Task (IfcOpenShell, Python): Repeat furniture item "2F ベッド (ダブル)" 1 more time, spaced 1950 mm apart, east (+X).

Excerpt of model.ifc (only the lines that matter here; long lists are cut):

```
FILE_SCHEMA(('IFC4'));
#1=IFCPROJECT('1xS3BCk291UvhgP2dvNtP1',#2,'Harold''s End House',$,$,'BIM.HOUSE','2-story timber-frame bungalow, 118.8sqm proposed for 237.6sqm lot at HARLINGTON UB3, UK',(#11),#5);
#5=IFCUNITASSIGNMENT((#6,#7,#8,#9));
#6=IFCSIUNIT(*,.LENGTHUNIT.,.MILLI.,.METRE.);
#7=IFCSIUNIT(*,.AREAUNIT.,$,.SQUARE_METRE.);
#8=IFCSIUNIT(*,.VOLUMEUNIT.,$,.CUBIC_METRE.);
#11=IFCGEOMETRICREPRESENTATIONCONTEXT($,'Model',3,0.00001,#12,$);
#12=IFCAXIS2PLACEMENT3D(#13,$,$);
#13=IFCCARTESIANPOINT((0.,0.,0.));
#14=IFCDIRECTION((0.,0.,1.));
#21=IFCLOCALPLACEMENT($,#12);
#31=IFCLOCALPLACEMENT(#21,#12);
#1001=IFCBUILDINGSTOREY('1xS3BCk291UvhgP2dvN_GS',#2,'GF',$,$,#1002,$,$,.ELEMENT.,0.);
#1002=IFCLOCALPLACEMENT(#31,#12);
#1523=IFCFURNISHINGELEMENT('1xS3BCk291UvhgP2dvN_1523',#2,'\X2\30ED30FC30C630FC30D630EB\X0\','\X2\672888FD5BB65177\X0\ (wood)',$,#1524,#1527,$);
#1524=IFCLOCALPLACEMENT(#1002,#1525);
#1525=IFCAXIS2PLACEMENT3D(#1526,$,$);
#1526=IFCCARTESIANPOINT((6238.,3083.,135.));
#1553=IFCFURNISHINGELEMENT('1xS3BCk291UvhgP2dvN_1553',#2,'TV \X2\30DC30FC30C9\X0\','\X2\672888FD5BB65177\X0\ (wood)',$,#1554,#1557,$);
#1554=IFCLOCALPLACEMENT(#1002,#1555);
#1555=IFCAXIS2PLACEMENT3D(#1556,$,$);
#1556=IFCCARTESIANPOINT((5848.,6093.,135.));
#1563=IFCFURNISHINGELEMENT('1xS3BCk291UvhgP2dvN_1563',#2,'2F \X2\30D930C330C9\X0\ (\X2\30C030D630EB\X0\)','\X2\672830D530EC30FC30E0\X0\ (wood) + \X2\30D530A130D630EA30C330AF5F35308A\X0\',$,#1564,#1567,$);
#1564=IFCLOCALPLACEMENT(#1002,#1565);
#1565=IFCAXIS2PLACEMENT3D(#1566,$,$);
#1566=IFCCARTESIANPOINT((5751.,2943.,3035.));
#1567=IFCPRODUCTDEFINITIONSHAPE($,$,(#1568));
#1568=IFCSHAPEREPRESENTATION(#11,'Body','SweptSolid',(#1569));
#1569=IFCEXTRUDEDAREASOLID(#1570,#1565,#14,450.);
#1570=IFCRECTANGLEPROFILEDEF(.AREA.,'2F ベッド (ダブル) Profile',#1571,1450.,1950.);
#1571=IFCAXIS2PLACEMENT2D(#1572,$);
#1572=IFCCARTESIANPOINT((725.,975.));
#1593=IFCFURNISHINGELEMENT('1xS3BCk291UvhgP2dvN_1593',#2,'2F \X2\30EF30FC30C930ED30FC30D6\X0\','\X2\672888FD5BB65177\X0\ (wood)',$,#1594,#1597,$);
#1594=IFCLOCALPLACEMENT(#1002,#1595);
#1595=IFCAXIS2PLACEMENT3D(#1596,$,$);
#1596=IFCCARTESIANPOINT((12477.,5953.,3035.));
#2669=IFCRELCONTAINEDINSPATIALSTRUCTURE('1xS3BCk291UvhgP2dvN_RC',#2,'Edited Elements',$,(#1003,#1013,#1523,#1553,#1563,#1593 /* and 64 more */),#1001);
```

```python
import numpy as np
import ifcopenshell
import ifcopenshell.api.geometry
import ifcopenshell.api.root
import ifcopenshell.util.element
import ifcopenshell.util.placement

model = ifcopenshell.open("model.ifc")


def reuse_history(source, copy):
    """copy_class also copies each property set's owner history, people and application; keep the originals."""
    for rel in copy.IsDefinedBy:
        if rel.is_a("IfcRelDefinesByProperties") and (history := rel.RelatingPropertyDefinition.OwnerHistory):
            rel.RelatingPropertyDefinition.OwnerHistory = source.OwnerHistory
            ifcopenshell.util.element.remove_deep2(model, history)


source = model.by_id(1563)
base = ifcopenshell.util.placement.get_local_placement(source.ObjectPlacement)
step = np.array([1.0, 0.0, 0.0]) * 1950.0

for i in range(1, 2):
    copy = ifcopenshell.api.root.copy_class(model, product=source)
    copy.Representation = ifcopenshell.util.element.copy_deep(
        model, source.Representation, exclude=["IfcGeometricRepresentationContext", "IfcRepresentationMap"]
    )
    reuse_history(source, copy)
    matrix = base.copy()
    matrix[:3, 3] += i * step
    print("added at", matrix[:3, 3].round(3) + 0.0)
    ifcopenshell.api.geometry.edit_object_placement(model, product=copy, matrix=matrix, is_si=False)

model.write("model_rev.ifc")
```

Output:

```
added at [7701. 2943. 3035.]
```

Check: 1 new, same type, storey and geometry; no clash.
